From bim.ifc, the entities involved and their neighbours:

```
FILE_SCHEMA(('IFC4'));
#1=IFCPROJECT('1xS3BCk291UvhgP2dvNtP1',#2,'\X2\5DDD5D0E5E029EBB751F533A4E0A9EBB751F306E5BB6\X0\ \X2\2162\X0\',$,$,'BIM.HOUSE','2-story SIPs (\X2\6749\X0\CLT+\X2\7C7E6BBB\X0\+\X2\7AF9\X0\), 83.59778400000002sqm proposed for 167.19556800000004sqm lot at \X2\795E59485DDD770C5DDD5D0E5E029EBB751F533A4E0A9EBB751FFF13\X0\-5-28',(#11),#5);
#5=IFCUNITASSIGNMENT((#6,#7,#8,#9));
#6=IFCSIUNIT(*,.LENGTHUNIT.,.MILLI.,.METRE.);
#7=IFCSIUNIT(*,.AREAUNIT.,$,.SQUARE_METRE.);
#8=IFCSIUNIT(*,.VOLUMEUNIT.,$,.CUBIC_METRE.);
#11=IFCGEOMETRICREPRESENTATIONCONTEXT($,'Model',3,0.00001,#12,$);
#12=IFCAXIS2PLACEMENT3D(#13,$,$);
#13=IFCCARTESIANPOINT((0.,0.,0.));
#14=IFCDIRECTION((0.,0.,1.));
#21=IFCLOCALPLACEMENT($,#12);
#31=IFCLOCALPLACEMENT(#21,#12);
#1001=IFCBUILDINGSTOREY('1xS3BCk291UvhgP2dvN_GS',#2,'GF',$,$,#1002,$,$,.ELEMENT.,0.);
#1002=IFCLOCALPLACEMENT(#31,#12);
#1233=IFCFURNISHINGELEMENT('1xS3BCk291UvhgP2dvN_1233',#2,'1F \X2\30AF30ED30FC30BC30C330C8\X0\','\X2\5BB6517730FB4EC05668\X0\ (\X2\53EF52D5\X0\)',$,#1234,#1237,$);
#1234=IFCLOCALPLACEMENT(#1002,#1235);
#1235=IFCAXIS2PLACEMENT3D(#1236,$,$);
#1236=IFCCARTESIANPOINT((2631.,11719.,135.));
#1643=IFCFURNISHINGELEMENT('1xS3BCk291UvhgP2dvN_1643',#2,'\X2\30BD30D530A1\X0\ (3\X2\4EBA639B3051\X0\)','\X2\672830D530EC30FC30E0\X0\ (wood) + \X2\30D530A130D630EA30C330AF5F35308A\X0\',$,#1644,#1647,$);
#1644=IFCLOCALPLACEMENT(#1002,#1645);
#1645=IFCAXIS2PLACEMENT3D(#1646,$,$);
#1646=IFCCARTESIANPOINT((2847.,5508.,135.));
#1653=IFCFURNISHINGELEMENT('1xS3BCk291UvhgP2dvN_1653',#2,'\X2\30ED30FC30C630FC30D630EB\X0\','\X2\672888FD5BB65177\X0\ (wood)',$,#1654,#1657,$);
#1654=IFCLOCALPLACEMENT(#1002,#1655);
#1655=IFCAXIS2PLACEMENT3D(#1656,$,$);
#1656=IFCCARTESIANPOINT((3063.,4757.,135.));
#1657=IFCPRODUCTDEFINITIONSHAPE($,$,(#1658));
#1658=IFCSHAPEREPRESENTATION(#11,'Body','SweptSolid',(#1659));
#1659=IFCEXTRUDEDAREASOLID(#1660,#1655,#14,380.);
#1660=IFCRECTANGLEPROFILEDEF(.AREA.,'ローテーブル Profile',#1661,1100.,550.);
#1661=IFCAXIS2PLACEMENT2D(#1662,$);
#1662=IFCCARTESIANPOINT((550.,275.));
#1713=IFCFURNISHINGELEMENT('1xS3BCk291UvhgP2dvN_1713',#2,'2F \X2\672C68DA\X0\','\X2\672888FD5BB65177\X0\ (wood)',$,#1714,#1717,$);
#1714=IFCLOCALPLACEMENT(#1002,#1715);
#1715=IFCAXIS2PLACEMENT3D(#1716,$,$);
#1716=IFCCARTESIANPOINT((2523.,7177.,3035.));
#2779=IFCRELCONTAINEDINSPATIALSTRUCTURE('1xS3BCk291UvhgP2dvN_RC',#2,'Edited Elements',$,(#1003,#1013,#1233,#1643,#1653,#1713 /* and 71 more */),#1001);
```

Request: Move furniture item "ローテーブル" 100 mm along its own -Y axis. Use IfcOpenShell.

```python
import ifcopenshell
import ifcopenshell.api.geometry
import ifcopenshell.util.placement
import ifcopenshell.util.unit

model = ifcopenshell.open("bim.ifc")
unit_scale = ifcopenshell.util.unit.calculate_unit_scale(model)

item = model.by_guid("1xS3BCk291UvhgP2dvN_1653")
matrix = ifcopenshell.util.placement.get_local_placement(item.ObjectPlacement)
matrix[:3, 3] -= matrix[:3, 1] * 0.1 / unit_scale
ifcopenshell.api.geometry.edit_object_placement(model, product=item, matrix=matrix, is_si=False)

print(ifcopenshell.util.placement.get_local_placement(item.ObjectPlacement).round(3) + 0.0)

model.write("bim_v2.ifc")
```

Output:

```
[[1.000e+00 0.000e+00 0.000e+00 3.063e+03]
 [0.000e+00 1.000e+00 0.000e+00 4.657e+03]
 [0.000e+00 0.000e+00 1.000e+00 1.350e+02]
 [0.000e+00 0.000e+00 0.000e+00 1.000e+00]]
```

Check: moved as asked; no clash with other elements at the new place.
